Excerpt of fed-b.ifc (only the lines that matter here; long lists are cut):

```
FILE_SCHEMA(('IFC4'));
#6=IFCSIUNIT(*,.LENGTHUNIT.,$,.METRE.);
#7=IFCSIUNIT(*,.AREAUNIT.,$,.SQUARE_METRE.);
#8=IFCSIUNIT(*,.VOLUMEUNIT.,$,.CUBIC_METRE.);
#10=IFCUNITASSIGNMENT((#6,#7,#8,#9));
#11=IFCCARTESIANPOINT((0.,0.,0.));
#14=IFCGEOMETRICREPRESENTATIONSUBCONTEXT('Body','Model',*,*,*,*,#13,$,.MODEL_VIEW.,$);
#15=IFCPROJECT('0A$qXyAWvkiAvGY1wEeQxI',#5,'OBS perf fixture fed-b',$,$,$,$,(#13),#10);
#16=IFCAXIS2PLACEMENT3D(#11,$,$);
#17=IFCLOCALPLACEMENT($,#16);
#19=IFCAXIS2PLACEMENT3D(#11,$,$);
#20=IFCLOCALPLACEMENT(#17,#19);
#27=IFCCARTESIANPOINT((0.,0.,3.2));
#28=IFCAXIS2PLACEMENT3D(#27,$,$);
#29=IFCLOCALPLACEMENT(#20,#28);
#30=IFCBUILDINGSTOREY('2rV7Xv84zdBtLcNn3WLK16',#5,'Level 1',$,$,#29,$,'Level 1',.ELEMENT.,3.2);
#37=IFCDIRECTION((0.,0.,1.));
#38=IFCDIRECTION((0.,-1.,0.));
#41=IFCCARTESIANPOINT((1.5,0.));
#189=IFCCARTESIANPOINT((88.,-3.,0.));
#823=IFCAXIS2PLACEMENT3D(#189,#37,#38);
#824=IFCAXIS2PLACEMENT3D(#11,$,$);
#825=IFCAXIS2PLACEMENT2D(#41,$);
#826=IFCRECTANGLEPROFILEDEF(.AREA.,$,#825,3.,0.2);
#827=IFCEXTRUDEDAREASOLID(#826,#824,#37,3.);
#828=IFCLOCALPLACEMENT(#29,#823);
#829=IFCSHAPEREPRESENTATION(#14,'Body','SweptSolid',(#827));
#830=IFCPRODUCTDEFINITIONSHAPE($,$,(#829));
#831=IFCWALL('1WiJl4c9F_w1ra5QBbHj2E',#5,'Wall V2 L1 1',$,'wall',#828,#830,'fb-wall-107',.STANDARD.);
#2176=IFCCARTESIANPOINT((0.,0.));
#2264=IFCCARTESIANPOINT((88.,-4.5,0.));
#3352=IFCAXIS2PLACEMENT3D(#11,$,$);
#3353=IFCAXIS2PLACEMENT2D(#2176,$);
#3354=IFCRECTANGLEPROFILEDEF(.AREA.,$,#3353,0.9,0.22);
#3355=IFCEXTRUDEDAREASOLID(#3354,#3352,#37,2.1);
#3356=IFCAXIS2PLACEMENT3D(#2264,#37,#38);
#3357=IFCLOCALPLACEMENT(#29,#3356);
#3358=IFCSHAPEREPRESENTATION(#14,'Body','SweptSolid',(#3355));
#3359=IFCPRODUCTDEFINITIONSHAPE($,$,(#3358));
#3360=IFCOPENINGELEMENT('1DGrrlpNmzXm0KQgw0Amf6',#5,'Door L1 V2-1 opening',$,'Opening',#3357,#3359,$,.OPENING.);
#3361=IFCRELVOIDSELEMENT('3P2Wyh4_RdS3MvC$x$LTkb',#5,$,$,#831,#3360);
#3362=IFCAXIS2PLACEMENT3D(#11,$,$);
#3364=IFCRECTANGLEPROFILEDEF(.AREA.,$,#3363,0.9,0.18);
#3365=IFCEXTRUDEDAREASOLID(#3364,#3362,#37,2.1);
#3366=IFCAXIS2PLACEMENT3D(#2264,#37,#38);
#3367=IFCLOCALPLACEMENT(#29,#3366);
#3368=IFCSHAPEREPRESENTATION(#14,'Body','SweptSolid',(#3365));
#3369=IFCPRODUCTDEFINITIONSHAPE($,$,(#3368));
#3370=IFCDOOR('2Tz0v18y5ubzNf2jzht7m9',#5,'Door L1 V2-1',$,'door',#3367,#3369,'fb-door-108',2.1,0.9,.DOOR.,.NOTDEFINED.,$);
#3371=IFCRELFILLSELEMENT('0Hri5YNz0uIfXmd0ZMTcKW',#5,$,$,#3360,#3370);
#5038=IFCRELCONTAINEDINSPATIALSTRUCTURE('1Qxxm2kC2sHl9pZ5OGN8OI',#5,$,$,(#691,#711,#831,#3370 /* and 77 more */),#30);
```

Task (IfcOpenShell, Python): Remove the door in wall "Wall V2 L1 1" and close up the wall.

```python
import ifcopenshell
import ifcopenshell.api.feature
import ifcopenshell.api.root
import ifcopenshell.geom
import ifcopenshell.util.shape

model = ifcopenshell.open("fed-b.ifc")
settings = ifcopenshell.geom.settings()


def volume(element):
    """Net volume in cubic metres, openings subtracted."""
    shape = ifcopenshell.geom.create_shape(settings, element)
    return ifcopenshell.util.shape.get_volume(shape.geometry)


door = model.by_guid("2Tz0v18y5ubzNf2jzht7m9")
opening = door.FillsVoids[0].RelatingOpeningElement
wall = opening.VoidsElements[0].RelatingBuildingElement
before = volume(wall)

ifcopenshell.api.root.remove_product(model, product=door)
ifcopenshell.api.feature.remove_feature(model, feature=opening)

after = volume(wall)

print(f"wall volume {before:.3f} -> {after:.3f} m3")

model.write("fed-b_edited.ifc")
```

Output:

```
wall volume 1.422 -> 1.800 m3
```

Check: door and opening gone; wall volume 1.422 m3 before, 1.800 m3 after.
